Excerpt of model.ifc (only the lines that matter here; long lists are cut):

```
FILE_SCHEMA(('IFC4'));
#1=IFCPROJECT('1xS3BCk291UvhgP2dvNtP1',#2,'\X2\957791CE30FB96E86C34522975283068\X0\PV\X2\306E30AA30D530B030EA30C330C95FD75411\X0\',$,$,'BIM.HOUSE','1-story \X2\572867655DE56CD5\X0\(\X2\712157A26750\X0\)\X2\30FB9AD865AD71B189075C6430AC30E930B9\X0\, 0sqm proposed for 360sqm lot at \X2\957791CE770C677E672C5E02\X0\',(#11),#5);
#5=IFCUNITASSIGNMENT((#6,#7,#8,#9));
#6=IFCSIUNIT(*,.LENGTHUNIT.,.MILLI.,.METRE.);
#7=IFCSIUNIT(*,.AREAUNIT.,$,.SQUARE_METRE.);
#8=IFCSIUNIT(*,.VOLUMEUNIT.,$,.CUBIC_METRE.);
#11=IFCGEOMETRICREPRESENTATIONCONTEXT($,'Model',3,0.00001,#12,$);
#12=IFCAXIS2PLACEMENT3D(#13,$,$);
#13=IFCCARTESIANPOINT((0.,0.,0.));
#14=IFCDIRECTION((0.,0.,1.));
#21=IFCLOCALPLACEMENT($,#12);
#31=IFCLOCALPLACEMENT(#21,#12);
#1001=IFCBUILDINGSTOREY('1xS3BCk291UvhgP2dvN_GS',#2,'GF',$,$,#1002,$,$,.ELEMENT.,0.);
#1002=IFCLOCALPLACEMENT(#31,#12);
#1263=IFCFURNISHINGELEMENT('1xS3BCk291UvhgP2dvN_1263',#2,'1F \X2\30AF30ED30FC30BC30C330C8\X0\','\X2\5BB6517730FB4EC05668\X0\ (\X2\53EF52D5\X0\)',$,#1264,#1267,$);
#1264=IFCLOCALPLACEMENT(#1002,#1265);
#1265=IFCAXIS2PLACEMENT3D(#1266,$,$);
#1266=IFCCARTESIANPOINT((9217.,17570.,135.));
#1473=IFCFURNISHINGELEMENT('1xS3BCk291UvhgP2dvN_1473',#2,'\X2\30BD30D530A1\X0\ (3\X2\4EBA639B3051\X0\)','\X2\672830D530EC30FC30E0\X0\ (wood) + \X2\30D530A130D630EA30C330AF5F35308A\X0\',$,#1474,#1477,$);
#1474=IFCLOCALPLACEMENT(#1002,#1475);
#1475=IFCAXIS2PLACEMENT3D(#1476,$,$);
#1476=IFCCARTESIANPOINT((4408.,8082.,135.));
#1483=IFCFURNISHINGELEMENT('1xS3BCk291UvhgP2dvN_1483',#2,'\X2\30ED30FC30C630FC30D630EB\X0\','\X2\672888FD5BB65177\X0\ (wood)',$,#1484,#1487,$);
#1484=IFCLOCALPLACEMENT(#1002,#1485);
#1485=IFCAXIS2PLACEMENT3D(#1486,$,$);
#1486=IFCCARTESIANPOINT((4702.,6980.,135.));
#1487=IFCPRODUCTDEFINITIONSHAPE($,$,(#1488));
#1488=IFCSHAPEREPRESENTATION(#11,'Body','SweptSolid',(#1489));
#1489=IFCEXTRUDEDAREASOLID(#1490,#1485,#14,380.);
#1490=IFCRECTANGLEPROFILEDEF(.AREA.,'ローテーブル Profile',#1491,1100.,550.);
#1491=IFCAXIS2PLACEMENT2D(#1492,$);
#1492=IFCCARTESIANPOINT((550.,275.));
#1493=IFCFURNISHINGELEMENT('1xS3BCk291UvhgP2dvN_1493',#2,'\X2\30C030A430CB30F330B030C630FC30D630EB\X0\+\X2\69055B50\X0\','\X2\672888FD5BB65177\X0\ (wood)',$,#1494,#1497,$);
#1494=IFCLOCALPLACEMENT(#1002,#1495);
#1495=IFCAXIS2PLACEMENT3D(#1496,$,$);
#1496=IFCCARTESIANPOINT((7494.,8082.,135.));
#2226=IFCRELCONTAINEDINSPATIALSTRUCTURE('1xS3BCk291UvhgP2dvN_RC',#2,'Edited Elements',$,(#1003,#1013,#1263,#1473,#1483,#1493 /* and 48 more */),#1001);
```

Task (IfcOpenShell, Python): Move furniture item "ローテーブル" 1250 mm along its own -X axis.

```python
import ifcopenshell
import ifcopenshell.api.geometry
import ifcopenshell.util.placement
import ifcopenshell.util.unit

model = ifcopenshell.open("model.ifc")
unit_scale = ifcopenshell.util.unit.calculate_unit_scale(model)

item = model.by_id(1483)
matrix = ifcopenshell.util.placement.get_local_placement(item.ObjectPlacement)
matrix[:3, 3] -= matrix[:3, 0] * 1.25 / unit_scale
ifcopenshell.api.geometry.edit_object_placement(model, product=item, matrix=matrix, is_si=False)

print(ifcopenshell.util.placement.get_local_placement(item.ObjectPlacement).round(3) + 0.0)

model.write("model_v2.ifc")
```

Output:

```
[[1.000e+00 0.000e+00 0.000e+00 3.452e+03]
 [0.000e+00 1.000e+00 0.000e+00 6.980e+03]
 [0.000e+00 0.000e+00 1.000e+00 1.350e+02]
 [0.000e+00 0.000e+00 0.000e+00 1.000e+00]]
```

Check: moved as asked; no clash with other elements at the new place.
